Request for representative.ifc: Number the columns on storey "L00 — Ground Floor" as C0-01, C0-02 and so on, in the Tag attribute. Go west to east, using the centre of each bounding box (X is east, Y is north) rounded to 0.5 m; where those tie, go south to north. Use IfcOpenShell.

First a look at what the model holds.

```python
import ifcopenshell
import ifcopenshell.util.element
import ifcopenshell.util.placement

model = ifcopenshell.open("representative.ifc")
print(model.schema)
storey = next(s for s in model.by_type("IfcBuildingStorey") if s.Name == "L00 — Ground Floor")
columns = [e for e in ifcopenshell.util.element.get_decomposition(storey) if e.is_a("IfcColumn")]
for e in sorted(columns, key=lambda e: e.id()):
    origin = ifcopenshell.util.placement.get_local_placement(e.ObjectPlacement)[:3, 3]
    print(e.id(), e.Tag, e.Name, origin.round(2) + 0.0, sep=" | ")
```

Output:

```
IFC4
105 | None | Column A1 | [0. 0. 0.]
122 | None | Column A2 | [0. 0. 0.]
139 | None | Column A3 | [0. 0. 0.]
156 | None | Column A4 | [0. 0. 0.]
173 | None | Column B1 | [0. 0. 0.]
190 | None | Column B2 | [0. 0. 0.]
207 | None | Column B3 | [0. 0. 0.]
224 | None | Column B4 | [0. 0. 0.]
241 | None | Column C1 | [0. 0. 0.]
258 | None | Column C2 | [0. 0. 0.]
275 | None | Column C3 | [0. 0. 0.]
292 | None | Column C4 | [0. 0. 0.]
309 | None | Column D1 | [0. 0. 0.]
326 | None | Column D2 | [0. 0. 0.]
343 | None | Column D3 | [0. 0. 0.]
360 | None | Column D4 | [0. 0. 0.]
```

```python
import ifcopenshell
import ifcopenshell.geom
import ifcopenshell.util.element
import ifcopenshell.util.shape

model = ifcopenshell.open("representative.ifc")
settings = ifcopenshell.geom.settings()
settings.set("use-world-coords", True)


def centre(element):
    shape = ifcopenshell.geom.create_shape(settings, element)
    return ifcopenshell.util.shape.get_bbox_centroid(shape.geometry)


storey = next(s for s in model.by_type("IfcBuildingStorey") if s.Name == "L00 — Ground Floor")
columns = [e for e in ifcopenshell.util.element.get_decomposition(storey) if e.is_a("IfcColumn")]

# Insertion points can sit at a corner or the storey origin, so sort by the geometry (in metres).
centres = {e: centre(e) for e in columns}
columns.sort(key=lambda e: (round(centres[e][0] / 0.5), centres[e][1]))

for i, e in enumerate(columns, start=1):
    number = f"C0-{i:02d}"
    e.Tag = number
    print(e.id(), number)

model.write("representative_rev.ifc")
```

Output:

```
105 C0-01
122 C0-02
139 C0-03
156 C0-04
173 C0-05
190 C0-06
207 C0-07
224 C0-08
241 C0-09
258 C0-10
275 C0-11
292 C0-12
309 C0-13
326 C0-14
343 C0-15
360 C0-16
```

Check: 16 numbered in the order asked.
